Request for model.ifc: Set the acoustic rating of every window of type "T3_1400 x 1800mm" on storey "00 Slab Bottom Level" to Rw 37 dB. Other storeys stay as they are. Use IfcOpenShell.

First a look at what the model holds.

```python
import ifcopenshell
import ifcopenshell.util.element

model = ifcopenshell.open("model.ifc")
print(model.schema)
storey = next(s for s in model.by_type("IfcBuildingStorey") if s.Name == "00 Slab Bottom Level")
windows = [e for e in ifcopenshell.util.element.get_decomposition(storey) if e.is_a("IfcWindow")]
seen = {}
for e in windows:
    element_type = ifcopenshell.util.element.get_type(e)
    key = (element_type.Name if element_type != e and element_type else None, ifcopenshell.util.element.get_pset(e, "Pset_WindowCommon", "AcousticRating"))
    seen[key] = seen.get(key, 0) + 1
for (name, value), count in sorted(seen.items(), key=str):
    print(count, "x", name, "|", value)
```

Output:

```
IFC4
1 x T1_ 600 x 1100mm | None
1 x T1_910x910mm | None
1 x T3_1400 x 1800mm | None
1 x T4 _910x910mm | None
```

```python
import ifcopenshell
import ifcopenshell.api.pset
import ifcopenshell.util.element

model = ifcopenshell.open("model.ifc")

storey = next(s for s in model.by_type("IfcBuildingStorey") if s.Name == "00 Slab Bottom Level")
windows = [e for e in ifcopenshell.util.element.get_decomposition(storey) if e.is_a("IfcWindow")]

count = 0
for e in windows:
    element_type = ifcopenshell.util.element.get_type(e)
    if element_type in (None, e) or element_type.Name != "T3_1400 x 1800mm":
        continue
    # add_pset returns the element's existing set when there is one.
    pset = ifcopenshell.api.pset.add_pset(model, product=e, name="Pset_WindowCommon")
    ifcopenshell.api.pset.edit_pset(model, pset=pset, properties={"AcousticRating": "Rw 37 dB"})
    count += 1

print(count, "windows updated")

model.write("model_v2.ifc")
```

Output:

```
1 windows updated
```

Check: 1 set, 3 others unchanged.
